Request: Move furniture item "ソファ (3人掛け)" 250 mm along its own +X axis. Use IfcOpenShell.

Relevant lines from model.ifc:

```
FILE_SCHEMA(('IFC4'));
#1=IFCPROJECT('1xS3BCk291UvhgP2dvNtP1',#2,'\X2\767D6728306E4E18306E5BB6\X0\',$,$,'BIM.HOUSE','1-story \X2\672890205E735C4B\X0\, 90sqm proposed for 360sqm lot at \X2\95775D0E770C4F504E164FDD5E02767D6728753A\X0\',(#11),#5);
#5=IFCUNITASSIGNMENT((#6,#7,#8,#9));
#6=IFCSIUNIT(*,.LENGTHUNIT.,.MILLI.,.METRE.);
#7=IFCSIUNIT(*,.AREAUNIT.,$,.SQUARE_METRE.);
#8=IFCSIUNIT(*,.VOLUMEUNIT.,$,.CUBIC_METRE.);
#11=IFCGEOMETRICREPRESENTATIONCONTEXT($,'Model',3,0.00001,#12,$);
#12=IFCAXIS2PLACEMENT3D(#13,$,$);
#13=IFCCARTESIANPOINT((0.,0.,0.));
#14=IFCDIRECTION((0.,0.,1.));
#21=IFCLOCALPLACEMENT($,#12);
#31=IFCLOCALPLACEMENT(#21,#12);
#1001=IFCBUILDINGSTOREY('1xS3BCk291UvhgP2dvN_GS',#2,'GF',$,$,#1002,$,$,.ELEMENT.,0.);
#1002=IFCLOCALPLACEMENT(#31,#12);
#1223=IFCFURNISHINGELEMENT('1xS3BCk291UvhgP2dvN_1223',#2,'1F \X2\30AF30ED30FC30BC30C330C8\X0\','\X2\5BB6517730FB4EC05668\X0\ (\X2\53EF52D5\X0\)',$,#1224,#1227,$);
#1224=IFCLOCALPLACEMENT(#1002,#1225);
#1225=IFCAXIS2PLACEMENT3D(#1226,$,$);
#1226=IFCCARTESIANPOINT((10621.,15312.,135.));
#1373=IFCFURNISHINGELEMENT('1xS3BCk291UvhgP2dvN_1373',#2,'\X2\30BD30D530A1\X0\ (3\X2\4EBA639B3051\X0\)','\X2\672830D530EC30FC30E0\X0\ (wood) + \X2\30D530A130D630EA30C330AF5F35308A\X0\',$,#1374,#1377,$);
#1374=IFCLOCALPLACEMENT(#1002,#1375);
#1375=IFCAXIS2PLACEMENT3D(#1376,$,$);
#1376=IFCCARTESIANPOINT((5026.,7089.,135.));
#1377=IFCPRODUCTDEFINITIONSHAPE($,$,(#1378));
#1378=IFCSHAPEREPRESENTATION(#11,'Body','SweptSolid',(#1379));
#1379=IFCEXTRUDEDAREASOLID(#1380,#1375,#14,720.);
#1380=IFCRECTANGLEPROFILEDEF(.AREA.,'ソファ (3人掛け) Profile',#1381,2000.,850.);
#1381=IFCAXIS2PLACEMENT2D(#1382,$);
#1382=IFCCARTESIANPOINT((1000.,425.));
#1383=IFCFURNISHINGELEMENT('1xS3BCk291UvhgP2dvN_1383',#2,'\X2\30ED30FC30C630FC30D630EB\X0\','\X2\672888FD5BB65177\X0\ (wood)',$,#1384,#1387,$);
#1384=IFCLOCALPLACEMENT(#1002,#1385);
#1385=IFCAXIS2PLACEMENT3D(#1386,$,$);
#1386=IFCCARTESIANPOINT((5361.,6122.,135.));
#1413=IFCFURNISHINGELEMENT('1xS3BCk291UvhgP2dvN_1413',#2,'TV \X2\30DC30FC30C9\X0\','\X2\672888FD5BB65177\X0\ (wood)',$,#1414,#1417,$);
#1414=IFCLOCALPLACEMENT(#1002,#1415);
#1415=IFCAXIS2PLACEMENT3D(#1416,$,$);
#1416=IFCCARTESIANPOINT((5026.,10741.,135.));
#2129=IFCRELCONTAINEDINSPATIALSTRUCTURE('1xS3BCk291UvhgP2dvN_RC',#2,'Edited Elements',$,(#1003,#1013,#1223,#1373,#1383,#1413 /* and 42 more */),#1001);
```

```python
import ifcopenshell
import ifcopenshell.api.geometry
import ifcopenshell.util.placement
import ifcopenshell.util.unit

model = ifcopenshell.open("model.ifc")
unit_scale = ifcopenshell.util.unit.calculate_unit_scale(model)

item = model.by_guid("1xS3BCk291UvhgP2dvN_1373")
matrix = ifcopenshell.util.placement.get_local_placement(item.ObjectPlacement)
matrix[:3, 3] += matrix[:3, 0] * 0.25 / unit_scale
ifcopenshell.api.geometry.edit_object_placement(model, product=item, matrix=matrix, is_si=False)

print(ifcopenshell.util.placement.get_local_placement(item.ObjectPlacement).round(3) + 0.0)

model.write("model_v2.ifc")
```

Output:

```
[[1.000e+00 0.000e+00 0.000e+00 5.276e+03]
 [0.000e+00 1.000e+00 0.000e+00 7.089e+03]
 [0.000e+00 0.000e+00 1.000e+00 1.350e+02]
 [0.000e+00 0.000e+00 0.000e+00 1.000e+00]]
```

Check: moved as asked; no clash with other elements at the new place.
